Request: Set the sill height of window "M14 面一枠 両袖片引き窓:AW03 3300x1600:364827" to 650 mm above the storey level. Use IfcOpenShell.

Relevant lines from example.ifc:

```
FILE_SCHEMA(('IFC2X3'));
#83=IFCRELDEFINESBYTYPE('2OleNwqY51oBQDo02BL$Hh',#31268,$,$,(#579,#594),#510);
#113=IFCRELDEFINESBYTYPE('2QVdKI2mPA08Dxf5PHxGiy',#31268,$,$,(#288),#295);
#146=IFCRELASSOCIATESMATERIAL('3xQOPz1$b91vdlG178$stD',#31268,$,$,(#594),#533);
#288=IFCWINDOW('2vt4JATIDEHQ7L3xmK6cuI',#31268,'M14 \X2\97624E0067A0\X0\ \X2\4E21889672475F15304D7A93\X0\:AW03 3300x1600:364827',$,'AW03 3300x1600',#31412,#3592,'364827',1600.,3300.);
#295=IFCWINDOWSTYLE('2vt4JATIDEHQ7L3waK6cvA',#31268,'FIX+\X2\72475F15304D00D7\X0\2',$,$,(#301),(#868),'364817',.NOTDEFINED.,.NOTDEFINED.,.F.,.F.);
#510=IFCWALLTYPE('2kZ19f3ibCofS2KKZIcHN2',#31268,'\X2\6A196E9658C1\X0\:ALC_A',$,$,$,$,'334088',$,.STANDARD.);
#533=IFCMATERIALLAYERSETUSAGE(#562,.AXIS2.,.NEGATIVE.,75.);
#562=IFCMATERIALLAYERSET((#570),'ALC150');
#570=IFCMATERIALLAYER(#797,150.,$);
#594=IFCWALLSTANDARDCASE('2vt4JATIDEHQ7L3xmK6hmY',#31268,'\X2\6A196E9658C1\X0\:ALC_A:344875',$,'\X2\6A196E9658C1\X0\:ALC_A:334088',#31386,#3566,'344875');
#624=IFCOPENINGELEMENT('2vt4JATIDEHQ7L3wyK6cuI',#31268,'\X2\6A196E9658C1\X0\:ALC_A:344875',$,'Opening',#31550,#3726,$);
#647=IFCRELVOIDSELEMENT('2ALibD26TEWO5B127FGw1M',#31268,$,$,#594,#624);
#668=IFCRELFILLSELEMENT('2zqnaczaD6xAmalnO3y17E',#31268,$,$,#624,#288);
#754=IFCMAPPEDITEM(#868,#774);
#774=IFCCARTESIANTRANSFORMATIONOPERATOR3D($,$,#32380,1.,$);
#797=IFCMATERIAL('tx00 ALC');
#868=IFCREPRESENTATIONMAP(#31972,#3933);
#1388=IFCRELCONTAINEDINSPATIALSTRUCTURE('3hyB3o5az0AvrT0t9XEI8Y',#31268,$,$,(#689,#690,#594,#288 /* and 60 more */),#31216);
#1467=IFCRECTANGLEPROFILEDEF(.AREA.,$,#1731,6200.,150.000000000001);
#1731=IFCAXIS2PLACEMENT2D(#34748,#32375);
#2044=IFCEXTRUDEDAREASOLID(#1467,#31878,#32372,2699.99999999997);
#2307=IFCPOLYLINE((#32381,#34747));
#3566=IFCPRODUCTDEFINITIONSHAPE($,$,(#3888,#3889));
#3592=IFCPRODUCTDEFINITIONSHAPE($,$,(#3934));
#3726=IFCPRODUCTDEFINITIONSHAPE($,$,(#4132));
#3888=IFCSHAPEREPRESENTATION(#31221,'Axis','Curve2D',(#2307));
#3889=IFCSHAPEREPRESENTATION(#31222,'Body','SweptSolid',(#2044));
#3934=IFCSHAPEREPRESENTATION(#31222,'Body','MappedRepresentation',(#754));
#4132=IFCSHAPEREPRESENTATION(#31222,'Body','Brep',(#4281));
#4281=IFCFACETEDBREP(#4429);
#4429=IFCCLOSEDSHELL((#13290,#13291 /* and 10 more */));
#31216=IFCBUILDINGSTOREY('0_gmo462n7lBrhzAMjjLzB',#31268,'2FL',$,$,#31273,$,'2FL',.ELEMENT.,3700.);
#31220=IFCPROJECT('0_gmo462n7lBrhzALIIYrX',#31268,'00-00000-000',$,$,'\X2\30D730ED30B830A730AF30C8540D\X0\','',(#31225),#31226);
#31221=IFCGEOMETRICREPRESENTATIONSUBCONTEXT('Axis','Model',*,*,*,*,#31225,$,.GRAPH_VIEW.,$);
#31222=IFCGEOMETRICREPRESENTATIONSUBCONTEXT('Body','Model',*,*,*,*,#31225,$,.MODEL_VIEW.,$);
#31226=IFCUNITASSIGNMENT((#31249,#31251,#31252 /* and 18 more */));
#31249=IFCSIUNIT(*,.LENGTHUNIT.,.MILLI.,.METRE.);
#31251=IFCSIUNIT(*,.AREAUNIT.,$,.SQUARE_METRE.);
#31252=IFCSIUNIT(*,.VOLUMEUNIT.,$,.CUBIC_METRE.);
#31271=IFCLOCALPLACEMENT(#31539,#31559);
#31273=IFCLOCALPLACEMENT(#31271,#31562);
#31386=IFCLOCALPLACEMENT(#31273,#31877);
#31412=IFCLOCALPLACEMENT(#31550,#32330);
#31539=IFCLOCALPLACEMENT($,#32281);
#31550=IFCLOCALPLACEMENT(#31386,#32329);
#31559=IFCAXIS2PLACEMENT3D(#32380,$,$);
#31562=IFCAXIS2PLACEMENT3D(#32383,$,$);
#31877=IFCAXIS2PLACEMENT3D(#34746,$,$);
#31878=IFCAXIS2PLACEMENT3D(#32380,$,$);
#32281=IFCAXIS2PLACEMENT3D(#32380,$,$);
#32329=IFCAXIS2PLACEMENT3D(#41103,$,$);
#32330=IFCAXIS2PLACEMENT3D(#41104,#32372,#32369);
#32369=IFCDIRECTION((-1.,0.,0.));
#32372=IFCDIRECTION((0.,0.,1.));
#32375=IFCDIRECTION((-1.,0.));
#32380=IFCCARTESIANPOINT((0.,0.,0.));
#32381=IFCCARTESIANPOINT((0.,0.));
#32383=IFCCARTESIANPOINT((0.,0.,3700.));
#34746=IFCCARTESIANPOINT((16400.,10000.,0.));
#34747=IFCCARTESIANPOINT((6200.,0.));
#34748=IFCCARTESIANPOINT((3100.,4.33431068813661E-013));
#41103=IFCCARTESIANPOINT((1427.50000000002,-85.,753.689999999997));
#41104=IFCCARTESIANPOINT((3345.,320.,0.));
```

```python
import numpy as np
import ifcopenshell
import ifcopenshell.api.geometry
import ifcopenshell.geom
import ifcopenshell.util.element
import ifcopenshell.util.placement
import ifcopenshell.util.shape
import ifcopenshell.util.unit

model = ifcopenshell.open("example.ifc")
unit_scale = ifcopenshell.util.unit.calculate_unit_scale(model)

window = model.by_guid("2vt4JATIDEHQ7L3xmK6cuI")
opening = window.FillsVoids[0].RelatingOpeningElement
storey = ifcopenshell.util.element.get_container(window, ifc_class="IfcBuildingStorey")
level = ifcopenshell.util.placement.get_local_placement(storey.ObjectPlacement)[2, 3]

# The opening's origin need not be at the sill, so measure its lowest point.
shape = ifcopenshell.geom.create_shape(ifcopenshell.geom.settings(), opening)
bottom = ifcopenshell.util.shape.get_shape_bottom_elevation(shape, shape.geometry) / unit_scale
dz = level + 0.65 / unit_scale - bottom

shift = np.array([0.0, 0.0, dz])
# The window is placed relative to its opening, so it follows when the opening moves.
matrix = ifcopenshell.util.placement.get_local_placement(opening.ObjectPlacement)
matrix[:3, 3] += shift
ifcopenshell.api.geometry.edit_object_placement(
    model, product=opening, matrix=matrix, is_si=False, should_transform_children=True
)

print(f"moved by {dz * unit_scale:+.3f} m")

model.write("example_updated.ifc")
```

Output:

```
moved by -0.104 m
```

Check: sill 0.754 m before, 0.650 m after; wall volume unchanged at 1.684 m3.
